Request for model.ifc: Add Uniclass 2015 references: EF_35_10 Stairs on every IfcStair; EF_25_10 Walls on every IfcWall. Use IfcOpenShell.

First a look at what the model holds.

```python
import ifcopenshell

model = ifcopenshell.open("model.ifc")
print(model.schema)
print("classifications:", [c.Name for c in model.by_type("IfcClassification")])
for ifc_class in ("IfcDoor", "IfcRoof", "IfcStair", "IfcWall", "IfcWindow"):
    print(ifc_class, len(model.by_type(ifc_class)))
```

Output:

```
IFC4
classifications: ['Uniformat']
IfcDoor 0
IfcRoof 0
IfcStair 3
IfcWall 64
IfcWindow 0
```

```python
import ifcopenshell
import ifcopenshell.api.classification

model = ifcopenshell.open("model.ifc")

system = ifcopenshell.api.classification.add_classification(model, classification="Uniclass 2015")

codes = {
    "IfcStair": ("EF_35_10", "Stairs"),
    "IfcWall": ("EF_25_10", "Walls"),
}
for ifc_class, (code, name) in codes.items():
    products = model.by_type(ifc_class)
    ifcopenshell.api.classification.add_reference(
        model, products=products, classification=system, identification=code, name=name
    )
    print(code, len(products))

model.write("model_v2.ifc")
```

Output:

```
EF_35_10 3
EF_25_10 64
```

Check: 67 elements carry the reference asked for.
